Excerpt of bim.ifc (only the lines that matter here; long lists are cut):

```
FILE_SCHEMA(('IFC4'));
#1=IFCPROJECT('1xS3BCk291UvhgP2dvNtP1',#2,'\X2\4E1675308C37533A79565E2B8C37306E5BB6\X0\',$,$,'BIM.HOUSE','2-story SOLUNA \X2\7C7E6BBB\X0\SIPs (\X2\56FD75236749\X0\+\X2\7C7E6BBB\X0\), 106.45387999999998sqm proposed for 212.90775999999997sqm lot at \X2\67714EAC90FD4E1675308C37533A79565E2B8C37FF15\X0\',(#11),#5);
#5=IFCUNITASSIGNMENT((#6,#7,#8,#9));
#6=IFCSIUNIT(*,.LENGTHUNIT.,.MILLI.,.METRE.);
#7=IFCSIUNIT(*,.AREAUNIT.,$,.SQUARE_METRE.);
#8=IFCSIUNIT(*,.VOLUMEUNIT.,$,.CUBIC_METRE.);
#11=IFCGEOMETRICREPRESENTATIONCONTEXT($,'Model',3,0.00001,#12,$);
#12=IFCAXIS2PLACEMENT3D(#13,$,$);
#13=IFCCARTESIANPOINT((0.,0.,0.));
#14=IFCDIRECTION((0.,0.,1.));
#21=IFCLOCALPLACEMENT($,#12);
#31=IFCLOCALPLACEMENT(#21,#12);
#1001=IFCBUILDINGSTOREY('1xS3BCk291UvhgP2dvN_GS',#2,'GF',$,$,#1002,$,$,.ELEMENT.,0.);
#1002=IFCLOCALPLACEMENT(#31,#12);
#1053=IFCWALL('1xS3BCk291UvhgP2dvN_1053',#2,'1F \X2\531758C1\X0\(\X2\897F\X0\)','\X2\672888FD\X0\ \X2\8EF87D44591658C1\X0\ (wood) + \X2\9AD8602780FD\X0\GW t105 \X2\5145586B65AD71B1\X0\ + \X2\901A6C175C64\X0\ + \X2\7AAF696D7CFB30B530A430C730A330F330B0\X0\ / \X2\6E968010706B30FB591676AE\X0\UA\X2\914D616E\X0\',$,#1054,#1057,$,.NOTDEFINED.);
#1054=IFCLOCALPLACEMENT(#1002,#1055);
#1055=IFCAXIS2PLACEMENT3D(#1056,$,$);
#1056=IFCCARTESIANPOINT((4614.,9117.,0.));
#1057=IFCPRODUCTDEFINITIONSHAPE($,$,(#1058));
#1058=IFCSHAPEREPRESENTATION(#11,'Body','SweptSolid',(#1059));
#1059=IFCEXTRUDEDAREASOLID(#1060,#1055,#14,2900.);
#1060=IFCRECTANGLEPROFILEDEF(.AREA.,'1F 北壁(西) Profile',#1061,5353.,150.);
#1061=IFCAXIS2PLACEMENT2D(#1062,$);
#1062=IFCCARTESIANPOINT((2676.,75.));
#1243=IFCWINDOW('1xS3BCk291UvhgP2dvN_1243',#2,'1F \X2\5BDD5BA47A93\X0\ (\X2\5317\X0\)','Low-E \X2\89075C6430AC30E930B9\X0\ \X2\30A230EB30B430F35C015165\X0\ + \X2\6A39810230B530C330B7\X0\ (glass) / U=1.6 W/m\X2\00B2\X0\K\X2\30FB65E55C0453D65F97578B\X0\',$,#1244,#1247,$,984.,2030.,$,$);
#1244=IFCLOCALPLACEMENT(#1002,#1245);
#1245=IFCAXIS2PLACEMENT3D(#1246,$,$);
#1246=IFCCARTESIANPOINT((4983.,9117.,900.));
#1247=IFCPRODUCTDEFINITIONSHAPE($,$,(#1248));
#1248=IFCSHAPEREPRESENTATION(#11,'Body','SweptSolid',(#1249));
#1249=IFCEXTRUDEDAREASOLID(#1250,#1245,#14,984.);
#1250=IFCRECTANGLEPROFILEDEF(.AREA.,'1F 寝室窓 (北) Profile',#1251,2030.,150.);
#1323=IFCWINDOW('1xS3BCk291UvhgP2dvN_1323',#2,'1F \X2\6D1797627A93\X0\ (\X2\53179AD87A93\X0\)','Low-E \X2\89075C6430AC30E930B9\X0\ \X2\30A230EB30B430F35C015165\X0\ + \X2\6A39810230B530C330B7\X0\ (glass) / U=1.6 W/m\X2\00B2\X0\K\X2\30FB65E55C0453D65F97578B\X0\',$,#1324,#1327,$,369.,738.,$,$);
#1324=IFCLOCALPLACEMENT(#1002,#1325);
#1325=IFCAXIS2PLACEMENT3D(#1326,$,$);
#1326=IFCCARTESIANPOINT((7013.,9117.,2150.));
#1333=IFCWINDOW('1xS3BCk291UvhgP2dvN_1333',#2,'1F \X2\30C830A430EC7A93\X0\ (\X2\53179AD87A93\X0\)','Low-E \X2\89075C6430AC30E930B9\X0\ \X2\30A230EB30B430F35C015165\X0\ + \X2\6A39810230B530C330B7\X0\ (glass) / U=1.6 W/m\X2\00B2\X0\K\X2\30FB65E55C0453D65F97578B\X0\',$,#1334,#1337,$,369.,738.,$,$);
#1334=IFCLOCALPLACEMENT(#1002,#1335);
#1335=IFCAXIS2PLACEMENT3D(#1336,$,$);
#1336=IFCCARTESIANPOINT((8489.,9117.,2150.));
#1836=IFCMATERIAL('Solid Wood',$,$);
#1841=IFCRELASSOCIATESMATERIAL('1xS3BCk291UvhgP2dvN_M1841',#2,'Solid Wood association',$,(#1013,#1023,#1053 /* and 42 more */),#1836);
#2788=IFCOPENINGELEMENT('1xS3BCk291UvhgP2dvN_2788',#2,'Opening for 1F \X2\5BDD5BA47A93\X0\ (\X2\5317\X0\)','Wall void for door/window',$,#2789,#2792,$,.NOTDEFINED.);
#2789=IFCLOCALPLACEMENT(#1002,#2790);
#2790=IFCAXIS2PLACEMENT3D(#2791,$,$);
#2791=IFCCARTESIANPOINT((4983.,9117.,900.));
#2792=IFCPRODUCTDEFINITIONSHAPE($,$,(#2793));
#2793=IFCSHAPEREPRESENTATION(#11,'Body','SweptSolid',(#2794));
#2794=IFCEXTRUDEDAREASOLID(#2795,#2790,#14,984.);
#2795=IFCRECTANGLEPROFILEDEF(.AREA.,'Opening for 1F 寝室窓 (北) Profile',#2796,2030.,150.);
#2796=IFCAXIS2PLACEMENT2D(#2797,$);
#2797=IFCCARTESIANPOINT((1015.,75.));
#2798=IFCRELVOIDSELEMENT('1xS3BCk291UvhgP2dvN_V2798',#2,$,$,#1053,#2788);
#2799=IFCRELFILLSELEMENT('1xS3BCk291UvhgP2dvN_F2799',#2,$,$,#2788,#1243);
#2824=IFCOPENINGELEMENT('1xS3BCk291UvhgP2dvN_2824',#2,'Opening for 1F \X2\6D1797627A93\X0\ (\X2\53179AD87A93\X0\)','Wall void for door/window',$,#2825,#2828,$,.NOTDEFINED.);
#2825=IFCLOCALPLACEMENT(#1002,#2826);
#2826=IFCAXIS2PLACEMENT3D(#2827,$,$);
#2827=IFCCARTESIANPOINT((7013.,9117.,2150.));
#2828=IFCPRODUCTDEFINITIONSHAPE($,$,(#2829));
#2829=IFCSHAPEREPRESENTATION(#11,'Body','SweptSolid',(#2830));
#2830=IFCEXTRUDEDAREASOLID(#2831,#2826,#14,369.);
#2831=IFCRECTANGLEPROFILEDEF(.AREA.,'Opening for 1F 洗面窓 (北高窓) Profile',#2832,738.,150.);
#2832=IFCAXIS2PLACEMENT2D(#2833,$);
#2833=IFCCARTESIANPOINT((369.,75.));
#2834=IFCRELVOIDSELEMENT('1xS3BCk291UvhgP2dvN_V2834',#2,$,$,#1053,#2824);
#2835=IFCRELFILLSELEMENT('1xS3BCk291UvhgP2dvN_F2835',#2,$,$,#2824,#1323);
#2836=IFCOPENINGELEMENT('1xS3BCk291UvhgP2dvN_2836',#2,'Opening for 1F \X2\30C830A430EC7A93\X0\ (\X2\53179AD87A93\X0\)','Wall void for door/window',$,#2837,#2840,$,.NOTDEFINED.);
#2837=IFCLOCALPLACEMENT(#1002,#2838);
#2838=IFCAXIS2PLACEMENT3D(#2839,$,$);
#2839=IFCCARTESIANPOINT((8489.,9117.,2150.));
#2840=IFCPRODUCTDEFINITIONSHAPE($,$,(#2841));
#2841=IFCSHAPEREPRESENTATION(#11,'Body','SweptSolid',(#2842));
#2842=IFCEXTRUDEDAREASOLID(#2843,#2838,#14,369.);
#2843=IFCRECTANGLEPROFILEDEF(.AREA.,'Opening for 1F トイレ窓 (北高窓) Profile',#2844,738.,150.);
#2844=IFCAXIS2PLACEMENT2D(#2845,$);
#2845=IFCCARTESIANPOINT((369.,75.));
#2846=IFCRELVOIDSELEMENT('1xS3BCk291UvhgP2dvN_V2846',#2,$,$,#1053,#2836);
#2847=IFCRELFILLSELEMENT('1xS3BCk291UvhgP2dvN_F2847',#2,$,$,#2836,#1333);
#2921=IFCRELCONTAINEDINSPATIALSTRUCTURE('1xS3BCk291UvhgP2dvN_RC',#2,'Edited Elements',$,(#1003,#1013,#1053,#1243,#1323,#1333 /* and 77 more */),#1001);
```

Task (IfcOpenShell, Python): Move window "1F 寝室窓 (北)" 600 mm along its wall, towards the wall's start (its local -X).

```python
import ifcopenshell
import ifcopenshell.api.geometry
import ifcopenshell.util.placement
import ifcopenshell.util.unit

model = ifcopenshell.open("bim.ifc")
unit_scale = ifcopenshell.util.unit.calculate_unit_scale(model)

window = model.by_id(1243)
opening = window.FillsVoids[0].RelatingOpeningElement
wall = opening.VoidsElements[0].RelatingBuildingElement

wall_matrix = ifcopenshell.util.placement.get_local_placement(wall.ObjectPlacement)
shift = wall_matrix[:3, 0] * -0.6 / unit_scale
before = ifcopenshell.util.placement.get_local_placement(window.ObjectPlacement)[:3, 3].copy()

# The window is not placed relative to its opening, so move both.
for product in (opening, window):
    matrix = ifcopenshell.util.placement.get_local_placement(product.ObjectPlacement)
    matrix[:3, 3] += shift
    ifcopenshell.api.geometry.edit_object_placement(model, product=product, matrix=matrix, is_si=False)

after = ifcopenshell.util.placement.get_local_placement(window.ObjectPlacement)[:3, 3]
print("window moved by", (after - before).round(3) + 0.0)

model.write("bim-out.ifc")
```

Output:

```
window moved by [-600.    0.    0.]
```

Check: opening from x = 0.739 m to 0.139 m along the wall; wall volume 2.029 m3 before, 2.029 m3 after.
